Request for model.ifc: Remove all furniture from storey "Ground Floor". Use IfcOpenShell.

First a look at what the model holds.

```python
import ifcopenshell
import ifcopenshell.util.element

model = ifcopenshell.open("model.ifc")
print(model.schema)
storey = next(s for s in model.by_type("IfcBuildingStorey") if s.Name == "Ground Floor")
furniture = [e for e in ifcopenshell.util.element.get_decomposition(storey) if e.is_a("IfcFurnishingElement")]
seen = {}
for e in furniture:
    element_type = ifcopenshell.util.element.get_type(e)
    name = element_type.Name if element_type not in (None, e) else None
    seen[name] = seen.get(name, 0) + 1
for name, count in sorted(seen.items(), key=str):
    print(count, "x", name)
```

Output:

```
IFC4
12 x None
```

```python
import ifcopenshell
import ifcopenshell.api.root
import ifcopenshell.util.element

model = ifcopenshell.open("model.ifc")

storey = next(s for s in model.by_type("IfcBuildingStorey") if s.Name == "Ground Floor")
furniture = [e for e in ifcopenshell.util.element.get_decomposition(storey) if e.is_a("IfcFurnishingElement")]

for e in furniture:
    ifcopenshell.api.root.remove_product(model, product=e)
print(len(furniture), "removed")

model.write("model_updated.ifc")
```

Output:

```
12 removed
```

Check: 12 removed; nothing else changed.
